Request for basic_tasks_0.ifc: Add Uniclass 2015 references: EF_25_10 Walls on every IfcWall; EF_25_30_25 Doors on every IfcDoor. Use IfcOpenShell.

First a look at what the model holds.

```python
import ifcopenshell

model = ifcopenshell.open("basic_tasks_0.ifc")
print(model.schema)
print("classifications:", [c.Name for c in model.by_type("IfcClassification")])
for ifc_class in ("IfcDoor", "IfcRoof", "IfcStair", "IfcWall", "IfcWindow"):
    print(ifc_class, len(model.by_type(ifc_class)))
```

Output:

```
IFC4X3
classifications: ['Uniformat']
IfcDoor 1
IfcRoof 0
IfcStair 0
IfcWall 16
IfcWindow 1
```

```python
import ifcopenshell
import ifcopenshell.api.classification

model = ifcopenshell.open("basic_tasks_0.ifc")

system = ifcopenshell.api.classification.add_classification(model, classification="Uniclass 2015")

codes = {
    "IfcWall": ("EF_25_10", "Walls"),
    "IfcDoor": ("EF_25_30_25", "Doors"),
}
for ifc_class, (code, name) in codes.items():
    products = model.by_type(ifc_class)
    ifcopenshell.api.classification.add_reference(
        model, products=products, classification=system, identification=code, name=name
    )
    print(code, len(products))

model.write("basic_tasks_0_updated.ifc")
```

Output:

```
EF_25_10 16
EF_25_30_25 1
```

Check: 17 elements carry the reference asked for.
